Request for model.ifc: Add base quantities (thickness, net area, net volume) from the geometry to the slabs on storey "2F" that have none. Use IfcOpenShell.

First a look at what the model holds.

```python
import ifcopenshell
import ifcopenshell.util.element
import ifcopenshell.util.unit

model = ifcopenshell.open("model.ifc")
print(model.schema)
for unit_type in ("LENGTHUNIT", "AREAUNIT", "VOLUMEUNIT"):
    print(unit_type, ifcopenshell.util.unit.calculate_unit_scale(model, unit_type))
storey = next(s for s in model.by_type("IfcBuildingStorey") if s.Name == "2F")
slabs = [e for e in ifcopenshell.util.element.get_decomposition(storey) if e.is_a("IfcSlab")]
for e in sorted(slabs, key=lambda e: e.id()):
    print(e.id(), e.is_a(), e.Name, list(ifcopenshell.util.element.get_psets(e, qtos_only=True)), sep=" | ")
```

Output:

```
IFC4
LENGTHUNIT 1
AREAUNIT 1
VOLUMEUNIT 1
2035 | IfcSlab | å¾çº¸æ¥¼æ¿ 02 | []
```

```python
import ifcopenshell
import ifcopenshell.api.pset
import ifcopenshell.geom
import ifcopenshell.util.element
import ifcopenshell.util.shape
import ifcopenshell.util.unit

model = ifcopenshell.open("model.ifc")
unit_scale = ifcopenshell.util.unit.calculate_unit_scale(model)
area_scale = ifcopenshell.util.unit.calculate_unit_scale(model, "AREAUNIT")
volume_scale = ifcopenshell.util.unit.calculate_unit_scale(model, "VOLUMEUNIT")
settings = ifcopenshell.geom.settings()

storey = next(s for s in model.by_type("IfcBuildingStorey") if s.Name == "2F")
slabs = [e for e in ifcopenshell.util.element.get_decomposition(storey) if e.is_a("IfcSlab")]

for e in sorted(slabs, key=lambda e: e.id()):
    if ifcopenshell.util.element.get_psets(e, qtos_only=True, should_inherit=False):
        continue
    # Geometry comes back in metres, in the element's own axes.
    shape = ifcopenshell.geom.create_shape(settings, e)
    values = {
        "Width": ifcopenshell.util.shape.get_z(shape.geometry) / unit_scale,
        "NetArea": ifcopenshell.util.shape.get_footprint_area(shape.geometry) / area_scale,
        "NetVolume": ifcopenshell.util.shape.get_volume(shape.geometry) / volume_scale,
    }
    qto = ifcopenshell.api.pset.add_qto(model, product=e, name="Qto_SlabBaseQuantities")
    ifcopenshell.api.pset.edit_qto(model, qto=qto, properties=values)
    print(e.id(), {k: round(v, 3) for k, v in values.items()})

model.write("model_edited.ifc")
```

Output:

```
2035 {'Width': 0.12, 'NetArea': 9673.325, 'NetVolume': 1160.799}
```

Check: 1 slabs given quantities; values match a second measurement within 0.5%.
